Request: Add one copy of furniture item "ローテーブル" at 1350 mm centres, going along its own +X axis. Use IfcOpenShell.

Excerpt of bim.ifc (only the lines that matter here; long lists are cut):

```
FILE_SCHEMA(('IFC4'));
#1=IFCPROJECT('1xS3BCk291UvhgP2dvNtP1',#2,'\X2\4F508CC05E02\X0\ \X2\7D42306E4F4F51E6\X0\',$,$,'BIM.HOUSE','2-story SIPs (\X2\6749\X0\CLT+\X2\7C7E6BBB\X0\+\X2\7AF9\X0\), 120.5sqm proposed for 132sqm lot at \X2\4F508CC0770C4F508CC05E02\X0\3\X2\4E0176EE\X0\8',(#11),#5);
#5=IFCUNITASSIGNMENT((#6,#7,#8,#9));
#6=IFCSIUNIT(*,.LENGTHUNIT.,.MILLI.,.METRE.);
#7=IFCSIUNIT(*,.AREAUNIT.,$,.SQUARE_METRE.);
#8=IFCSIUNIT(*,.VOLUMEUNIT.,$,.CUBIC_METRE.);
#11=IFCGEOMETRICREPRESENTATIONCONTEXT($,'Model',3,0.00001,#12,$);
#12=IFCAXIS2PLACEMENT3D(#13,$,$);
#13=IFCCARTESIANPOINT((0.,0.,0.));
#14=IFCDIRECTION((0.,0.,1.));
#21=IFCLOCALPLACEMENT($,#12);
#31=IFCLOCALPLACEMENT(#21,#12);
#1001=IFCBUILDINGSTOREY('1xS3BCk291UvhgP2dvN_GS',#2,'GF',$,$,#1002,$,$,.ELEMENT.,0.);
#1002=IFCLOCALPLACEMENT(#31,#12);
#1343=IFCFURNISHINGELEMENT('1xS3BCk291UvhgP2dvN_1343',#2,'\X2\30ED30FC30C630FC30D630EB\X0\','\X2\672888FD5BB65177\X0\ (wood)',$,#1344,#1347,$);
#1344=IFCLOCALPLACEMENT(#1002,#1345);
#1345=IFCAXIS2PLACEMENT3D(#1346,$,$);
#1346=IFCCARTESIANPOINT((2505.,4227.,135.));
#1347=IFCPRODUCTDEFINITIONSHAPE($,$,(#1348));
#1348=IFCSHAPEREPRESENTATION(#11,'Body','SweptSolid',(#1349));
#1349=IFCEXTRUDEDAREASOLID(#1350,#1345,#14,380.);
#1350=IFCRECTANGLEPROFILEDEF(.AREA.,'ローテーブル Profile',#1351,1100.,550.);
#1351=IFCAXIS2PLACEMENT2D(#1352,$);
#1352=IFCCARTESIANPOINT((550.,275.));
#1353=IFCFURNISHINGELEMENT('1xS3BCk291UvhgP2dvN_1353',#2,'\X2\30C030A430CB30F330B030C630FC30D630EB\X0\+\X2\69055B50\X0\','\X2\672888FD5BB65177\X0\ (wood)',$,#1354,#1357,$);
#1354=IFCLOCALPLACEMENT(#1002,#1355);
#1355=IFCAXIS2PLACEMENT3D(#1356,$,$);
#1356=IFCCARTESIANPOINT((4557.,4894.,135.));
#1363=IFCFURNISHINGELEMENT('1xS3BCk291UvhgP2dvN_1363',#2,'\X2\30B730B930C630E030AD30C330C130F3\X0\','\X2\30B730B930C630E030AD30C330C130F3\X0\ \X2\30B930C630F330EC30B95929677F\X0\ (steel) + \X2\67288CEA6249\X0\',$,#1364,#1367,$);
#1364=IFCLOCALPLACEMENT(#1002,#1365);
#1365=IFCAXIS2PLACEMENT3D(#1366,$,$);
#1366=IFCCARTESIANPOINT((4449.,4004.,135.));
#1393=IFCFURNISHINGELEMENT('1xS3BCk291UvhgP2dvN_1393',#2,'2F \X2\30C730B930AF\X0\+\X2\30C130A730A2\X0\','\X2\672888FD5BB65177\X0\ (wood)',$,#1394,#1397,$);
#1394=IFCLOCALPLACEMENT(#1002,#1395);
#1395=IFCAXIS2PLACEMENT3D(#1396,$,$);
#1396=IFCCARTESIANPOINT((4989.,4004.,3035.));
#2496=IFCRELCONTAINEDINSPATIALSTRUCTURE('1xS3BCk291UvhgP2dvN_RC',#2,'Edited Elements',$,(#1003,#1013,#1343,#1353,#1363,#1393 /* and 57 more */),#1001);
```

```python
import ifcopenshell
import ifcopenshell.api.geometry
import ifcopenshell.api.root
import ifcopenshell.util.element
import ifcopenshell.util.placement
import ifcopenshell.util.unit

model = ifcopenshell.open("bim.ifc")
unit_scale = ifcopenshell.util.unit.calculate_unit_scale(model)


def reuse_history(source, copy):
    """copy_class also copies each property set's owner history, people and application; keep the originals."""
    for rel in copy.IsDefinedBy:
        if rel.is_a("IfcRelDefinesByProperties") and (history := rel.RelatingPropertyDefinition.OwnerHistory):
            rel.RelatingPropertyDefinition.OwnerHistory = source.OwnerHistory
            ifcopenshell.util.element.remove_deep2(model, history)


source = model.by_guid("1xS3BCk291UvhgP2dvN_1343")
base = ifcopenshell.util.placement.get_local_placement(source.ObjectPlacement)
step = base[:3, 0] * 1.35 / unit_scale

for i in range(1, 2):
    copy = ifcopenshell.api.root.copy_class(model, product=source)
    copy.Representation = ifcopenshell.util.element.copy_deep(
        model, source.Representation, exclude=["IfcGeometricRepresentationContext", "IfcRepresentationMap"]
    )
    reuse_history(source, copy)
    matrix = base.copy()
    matrix[:3, 3] += i * step
    print("added at", matrix[:3, 3].round(3) + 0.0)
    ifcopenshell.api.geometry.edit_object_placement(model, product=copy, matrix=matrix, is_si=False)

model.write("bim_v2.ifc")
```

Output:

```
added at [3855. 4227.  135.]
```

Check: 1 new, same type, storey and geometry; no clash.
